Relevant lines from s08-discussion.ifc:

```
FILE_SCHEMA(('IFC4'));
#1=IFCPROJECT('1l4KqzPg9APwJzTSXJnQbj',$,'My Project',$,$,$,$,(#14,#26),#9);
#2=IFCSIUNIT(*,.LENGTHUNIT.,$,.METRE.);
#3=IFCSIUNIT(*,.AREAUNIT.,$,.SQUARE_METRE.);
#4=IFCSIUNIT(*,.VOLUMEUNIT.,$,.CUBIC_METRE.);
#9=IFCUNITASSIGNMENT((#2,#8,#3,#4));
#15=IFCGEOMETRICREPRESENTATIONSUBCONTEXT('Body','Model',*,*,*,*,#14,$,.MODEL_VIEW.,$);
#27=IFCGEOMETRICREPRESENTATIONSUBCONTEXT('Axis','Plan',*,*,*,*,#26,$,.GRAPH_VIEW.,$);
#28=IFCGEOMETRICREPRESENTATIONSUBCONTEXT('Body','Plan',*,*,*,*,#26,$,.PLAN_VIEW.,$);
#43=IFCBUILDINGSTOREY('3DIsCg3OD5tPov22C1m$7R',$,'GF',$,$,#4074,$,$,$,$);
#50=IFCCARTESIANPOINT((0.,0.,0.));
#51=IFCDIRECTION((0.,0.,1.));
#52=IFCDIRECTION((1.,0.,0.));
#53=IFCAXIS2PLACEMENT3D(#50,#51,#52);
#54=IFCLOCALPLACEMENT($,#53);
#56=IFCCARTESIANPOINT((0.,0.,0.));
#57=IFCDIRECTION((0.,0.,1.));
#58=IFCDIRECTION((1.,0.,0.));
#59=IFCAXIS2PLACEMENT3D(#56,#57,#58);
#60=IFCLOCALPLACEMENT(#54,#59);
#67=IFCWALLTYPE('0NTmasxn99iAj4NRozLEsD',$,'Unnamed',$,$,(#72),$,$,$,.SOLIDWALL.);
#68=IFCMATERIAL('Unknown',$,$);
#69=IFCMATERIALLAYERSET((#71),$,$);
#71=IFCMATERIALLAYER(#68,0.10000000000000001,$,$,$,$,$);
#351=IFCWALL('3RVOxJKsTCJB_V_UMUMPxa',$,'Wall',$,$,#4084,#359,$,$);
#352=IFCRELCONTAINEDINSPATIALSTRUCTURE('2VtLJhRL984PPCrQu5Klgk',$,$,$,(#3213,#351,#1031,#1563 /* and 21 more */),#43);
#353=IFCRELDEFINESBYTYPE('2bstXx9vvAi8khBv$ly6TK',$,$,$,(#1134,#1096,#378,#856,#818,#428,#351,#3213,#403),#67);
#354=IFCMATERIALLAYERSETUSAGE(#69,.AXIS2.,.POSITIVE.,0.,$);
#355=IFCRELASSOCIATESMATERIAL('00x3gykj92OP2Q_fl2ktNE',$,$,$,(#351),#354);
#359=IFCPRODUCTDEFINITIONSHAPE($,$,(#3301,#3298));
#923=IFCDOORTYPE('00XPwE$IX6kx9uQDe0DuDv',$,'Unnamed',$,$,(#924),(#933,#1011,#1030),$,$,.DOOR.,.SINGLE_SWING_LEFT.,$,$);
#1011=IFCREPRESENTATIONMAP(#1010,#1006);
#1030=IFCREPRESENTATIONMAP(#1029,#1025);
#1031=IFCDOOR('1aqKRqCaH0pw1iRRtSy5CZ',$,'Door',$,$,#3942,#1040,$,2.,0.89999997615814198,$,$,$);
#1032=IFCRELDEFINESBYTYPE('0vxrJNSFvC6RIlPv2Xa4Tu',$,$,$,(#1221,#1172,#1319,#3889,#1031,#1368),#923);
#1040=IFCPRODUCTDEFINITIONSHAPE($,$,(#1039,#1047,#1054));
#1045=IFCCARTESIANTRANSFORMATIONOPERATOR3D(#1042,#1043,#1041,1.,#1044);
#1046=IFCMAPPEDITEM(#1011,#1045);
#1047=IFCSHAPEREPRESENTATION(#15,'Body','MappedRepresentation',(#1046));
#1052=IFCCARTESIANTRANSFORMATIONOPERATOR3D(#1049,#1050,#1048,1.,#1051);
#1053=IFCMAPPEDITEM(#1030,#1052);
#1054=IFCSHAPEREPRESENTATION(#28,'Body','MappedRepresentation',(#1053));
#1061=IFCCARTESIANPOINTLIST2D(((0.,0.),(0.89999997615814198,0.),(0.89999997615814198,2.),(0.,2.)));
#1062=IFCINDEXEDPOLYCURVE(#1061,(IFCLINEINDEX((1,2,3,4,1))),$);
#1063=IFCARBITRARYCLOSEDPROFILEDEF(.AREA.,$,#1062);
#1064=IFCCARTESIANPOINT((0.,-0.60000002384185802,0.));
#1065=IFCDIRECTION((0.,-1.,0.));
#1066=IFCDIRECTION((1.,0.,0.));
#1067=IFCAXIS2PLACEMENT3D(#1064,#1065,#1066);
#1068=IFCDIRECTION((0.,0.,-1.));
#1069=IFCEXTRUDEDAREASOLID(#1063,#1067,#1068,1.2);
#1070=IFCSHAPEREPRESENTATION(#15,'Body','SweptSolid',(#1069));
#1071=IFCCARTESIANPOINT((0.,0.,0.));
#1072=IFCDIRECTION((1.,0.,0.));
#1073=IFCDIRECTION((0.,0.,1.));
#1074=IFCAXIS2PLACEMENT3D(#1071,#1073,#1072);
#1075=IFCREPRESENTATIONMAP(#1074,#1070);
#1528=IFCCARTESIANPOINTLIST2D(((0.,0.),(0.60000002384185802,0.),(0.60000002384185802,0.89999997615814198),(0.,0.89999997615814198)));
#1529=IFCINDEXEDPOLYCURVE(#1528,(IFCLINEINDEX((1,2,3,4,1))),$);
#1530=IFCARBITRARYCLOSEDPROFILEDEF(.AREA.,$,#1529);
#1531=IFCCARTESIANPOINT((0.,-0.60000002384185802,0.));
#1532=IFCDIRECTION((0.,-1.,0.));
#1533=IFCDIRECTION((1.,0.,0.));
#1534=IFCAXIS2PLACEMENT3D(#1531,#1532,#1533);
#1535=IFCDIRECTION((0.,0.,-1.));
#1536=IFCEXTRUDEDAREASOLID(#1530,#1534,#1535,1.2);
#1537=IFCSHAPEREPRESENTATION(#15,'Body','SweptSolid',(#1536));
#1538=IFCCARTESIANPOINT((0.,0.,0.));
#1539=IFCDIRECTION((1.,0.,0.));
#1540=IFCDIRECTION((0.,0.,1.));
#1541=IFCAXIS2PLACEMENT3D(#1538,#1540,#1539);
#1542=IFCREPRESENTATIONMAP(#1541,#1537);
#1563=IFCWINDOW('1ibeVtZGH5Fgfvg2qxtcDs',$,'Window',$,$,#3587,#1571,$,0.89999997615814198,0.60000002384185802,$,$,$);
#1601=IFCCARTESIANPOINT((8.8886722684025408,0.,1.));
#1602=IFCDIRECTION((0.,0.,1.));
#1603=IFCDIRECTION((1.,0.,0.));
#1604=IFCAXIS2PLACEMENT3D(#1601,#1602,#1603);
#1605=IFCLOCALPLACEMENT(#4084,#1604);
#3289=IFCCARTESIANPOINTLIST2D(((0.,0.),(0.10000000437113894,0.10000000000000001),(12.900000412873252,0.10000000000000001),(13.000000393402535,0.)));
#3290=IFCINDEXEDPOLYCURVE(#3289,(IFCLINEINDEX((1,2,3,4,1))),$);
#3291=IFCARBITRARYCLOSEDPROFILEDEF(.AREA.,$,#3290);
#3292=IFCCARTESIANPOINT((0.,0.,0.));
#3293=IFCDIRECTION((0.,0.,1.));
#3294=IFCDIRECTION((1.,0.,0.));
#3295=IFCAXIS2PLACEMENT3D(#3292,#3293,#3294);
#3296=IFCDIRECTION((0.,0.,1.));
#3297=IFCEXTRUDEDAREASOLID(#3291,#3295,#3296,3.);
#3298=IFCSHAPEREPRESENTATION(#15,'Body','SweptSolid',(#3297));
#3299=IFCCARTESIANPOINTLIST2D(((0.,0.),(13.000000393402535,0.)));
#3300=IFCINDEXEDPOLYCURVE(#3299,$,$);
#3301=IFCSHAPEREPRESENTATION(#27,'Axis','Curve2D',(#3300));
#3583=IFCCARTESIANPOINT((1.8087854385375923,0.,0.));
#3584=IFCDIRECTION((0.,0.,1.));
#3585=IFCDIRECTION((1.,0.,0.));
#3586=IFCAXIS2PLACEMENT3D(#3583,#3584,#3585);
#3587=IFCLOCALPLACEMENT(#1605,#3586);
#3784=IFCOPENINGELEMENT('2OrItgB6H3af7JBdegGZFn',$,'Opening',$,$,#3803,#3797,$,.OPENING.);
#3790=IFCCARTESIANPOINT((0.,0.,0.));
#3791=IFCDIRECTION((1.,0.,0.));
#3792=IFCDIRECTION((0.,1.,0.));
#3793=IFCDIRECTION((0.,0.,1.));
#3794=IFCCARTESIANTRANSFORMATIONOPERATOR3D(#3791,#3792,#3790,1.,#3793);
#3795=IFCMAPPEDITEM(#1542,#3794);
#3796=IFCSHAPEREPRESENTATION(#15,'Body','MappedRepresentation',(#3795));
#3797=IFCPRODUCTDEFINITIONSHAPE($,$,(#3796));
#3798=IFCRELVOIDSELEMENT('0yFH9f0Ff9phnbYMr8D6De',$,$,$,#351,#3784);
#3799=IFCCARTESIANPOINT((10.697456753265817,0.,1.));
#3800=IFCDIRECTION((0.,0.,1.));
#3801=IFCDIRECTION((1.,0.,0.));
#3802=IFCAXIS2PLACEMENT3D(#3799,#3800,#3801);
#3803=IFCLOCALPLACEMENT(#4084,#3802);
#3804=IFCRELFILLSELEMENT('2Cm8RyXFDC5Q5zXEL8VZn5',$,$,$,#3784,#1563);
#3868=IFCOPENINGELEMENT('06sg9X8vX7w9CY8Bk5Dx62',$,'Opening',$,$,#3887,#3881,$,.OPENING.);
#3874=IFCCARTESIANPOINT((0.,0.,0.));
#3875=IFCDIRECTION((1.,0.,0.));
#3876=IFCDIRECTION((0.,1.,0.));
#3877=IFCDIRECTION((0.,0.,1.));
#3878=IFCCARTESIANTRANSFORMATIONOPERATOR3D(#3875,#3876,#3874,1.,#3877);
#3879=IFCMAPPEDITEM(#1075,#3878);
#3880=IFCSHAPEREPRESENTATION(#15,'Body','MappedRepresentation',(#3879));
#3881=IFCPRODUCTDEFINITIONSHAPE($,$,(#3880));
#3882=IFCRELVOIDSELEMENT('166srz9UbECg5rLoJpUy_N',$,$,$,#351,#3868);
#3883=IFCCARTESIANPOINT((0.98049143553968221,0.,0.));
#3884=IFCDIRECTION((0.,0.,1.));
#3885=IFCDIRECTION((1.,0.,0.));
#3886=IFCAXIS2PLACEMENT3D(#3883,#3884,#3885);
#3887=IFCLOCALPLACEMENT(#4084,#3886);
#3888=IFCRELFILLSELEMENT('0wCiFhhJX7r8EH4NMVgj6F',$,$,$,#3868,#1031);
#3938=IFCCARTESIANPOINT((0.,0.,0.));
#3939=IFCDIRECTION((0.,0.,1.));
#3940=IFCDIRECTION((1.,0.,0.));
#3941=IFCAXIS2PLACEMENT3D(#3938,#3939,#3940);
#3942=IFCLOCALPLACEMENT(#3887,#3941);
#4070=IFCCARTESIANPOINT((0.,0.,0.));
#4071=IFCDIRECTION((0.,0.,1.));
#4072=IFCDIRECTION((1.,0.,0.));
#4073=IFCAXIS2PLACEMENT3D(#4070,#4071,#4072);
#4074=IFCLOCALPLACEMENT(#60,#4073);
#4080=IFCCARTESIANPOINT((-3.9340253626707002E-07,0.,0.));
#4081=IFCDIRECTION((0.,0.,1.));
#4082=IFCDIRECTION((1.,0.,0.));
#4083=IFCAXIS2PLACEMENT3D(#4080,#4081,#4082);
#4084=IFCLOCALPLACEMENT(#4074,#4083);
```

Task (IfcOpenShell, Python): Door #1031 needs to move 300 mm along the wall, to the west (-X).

```python
import ifcopenshell
import ifcopenshell.api.geometry
import ifcopenshell.util.placement

model = ifcopenshell.open("s08-discussion.ifc")

door = model.by_guid("1aqKRqCaH0pw1iRRtSy5CZ")
opening = door.FillsVoids[0].RelatingOpeningElement
wall = opening.VoidsElements[0].RelatingBuildingElement

wall_matrix = ifcopenshell.util.placement.get_local_placement(wall.ObjectPlacement)
shift = wall_matrix[:3, 0] * -0.3
before = ifcopenshell.util.placement.get_local_placement(door.ObjectPlacement)[:3, 3].copy()

# The door is placed relative to its opening, so it follows when the opening moves.
matrix = ifcopenshell.util.placement.get_local_placement(opening.ObjectPlacement)
matrix[:3, 3] += shift
ifcopenshell.api.geometry.edit_object_placement(
    model, product=opening, matrix=matrix, is_si=False, should_transform_children=True
)

after = ifcopenshell.util.placement.get_local_placement(door.ObjectPlacement)[:3, 3]
print("door moved by", (after - before).round(3) + 0.0)

model.write("s08-discussion_updated.ifc")
```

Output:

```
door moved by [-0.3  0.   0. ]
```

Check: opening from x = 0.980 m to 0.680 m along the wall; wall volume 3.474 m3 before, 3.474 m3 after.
